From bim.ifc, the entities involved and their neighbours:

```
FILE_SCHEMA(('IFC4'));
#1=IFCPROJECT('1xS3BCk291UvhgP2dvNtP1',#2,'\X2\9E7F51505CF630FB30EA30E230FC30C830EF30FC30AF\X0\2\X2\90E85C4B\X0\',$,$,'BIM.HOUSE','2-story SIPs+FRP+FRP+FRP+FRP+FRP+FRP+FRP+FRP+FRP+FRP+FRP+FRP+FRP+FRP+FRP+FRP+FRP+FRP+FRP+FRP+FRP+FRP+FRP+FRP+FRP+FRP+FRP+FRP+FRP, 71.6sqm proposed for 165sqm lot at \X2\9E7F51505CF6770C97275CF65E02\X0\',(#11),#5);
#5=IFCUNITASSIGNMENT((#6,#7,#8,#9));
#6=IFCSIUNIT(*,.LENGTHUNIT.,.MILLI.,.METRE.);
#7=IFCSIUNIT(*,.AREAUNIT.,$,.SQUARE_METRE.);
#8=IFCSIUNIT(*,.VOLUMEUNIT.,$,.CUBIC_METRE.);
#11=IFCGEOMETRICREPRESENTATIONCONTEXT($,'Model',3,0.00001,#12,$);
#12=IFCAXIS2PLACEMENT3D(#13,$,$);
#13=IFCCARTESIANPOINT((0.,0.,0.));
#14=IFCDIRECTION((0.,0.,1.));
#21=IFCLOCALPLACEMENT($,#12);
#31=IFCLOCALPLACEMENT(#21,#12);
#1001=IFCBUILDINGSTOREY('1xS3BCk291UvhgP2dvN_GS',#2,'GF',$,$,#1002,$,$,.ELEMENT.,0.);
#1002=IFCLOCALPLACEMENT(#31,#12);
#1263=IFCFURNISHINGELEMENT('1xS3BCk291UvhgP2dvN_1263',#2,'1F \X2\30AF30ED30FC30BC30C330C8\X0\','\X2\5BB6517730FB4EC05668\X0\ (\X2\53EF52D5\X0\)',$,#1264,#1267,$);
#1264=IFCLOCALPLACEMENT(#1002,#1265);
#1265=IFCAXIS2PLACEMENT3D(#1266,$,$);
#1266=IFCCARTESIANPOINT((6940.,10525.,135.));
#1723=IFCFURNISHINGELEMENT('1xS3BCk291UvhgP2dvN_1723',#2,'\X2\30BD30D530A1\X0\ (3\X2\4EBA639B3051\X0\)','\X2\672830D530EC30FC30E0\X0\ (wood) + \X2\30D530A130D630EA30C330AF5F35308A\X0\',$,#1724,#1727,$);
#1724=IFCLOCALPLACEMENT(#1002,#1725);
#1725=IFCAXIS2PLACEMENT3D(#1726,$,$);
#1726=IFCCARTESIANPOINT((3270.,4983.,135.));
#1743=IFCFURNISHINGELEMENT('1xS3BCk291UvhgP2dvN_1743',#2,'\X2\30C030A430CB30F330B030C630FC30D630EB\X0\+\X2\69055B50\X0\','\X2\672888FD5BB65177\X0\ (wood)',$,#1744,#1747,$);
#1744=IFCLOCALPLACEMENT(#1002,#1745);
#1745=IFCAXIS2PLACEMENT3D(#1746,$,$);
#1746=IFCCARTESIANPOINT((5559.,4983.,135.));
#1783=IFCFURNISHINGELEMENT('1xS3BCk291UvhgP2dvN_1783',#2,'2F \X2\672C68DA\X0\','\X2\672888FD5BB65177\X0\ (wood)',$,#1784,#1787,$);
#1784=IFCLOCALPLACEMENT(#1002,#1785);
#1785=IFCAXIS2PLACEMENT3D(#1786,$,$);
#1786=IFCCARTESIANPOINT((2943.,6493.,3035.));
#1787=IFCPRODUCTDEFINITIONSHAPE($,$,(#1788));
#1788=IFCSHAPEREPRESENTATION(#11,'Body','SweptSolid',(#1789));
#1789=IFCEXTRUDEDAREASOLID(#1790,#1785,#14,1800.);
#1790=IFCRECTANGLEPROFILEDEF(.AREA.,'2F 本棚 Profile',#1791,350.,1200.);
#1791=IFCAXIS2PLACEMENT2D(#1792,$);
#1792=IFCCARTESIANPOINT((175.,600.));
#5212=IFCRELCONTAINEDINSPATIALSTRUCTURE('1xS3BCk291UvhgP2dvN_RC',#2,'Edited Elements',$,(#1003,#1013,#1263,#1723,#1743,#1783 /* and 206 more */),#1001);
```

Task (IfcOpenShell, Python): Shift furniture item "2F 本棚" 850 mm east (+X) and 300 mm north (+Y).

```python
import ifcopenshell
import ifcopenshell.api.geometry
import ifcopenshell.util.placement

model = ifcopenshell.open("bim.ifc")

item = model.by_guid("1xS3BCk291UvhgP2dvN_1783")
matrix = ifcopenshell.util.placement.get_local_placement(item.ObjectPlacement)
matrix[0, 3] += 850.0
matrix[1, 3] += 300.0
ifcopenshell.api.geometry.edit_object_placement(model, product=item, matrix=matrix, is_si=False)

print(ifcopenshell.util.placement.get_local_placement(item.ObjectPlacement).round(3) + 0.0)

model.write("bim_updated.ifc")
```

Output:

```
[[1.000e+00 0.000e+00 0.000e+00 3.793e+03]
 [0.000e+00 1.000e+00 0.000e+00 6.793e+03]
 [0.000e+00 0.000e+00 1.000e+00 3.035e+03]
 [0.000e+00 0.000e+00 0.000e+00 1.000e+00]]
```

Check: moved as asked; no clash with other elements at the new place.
